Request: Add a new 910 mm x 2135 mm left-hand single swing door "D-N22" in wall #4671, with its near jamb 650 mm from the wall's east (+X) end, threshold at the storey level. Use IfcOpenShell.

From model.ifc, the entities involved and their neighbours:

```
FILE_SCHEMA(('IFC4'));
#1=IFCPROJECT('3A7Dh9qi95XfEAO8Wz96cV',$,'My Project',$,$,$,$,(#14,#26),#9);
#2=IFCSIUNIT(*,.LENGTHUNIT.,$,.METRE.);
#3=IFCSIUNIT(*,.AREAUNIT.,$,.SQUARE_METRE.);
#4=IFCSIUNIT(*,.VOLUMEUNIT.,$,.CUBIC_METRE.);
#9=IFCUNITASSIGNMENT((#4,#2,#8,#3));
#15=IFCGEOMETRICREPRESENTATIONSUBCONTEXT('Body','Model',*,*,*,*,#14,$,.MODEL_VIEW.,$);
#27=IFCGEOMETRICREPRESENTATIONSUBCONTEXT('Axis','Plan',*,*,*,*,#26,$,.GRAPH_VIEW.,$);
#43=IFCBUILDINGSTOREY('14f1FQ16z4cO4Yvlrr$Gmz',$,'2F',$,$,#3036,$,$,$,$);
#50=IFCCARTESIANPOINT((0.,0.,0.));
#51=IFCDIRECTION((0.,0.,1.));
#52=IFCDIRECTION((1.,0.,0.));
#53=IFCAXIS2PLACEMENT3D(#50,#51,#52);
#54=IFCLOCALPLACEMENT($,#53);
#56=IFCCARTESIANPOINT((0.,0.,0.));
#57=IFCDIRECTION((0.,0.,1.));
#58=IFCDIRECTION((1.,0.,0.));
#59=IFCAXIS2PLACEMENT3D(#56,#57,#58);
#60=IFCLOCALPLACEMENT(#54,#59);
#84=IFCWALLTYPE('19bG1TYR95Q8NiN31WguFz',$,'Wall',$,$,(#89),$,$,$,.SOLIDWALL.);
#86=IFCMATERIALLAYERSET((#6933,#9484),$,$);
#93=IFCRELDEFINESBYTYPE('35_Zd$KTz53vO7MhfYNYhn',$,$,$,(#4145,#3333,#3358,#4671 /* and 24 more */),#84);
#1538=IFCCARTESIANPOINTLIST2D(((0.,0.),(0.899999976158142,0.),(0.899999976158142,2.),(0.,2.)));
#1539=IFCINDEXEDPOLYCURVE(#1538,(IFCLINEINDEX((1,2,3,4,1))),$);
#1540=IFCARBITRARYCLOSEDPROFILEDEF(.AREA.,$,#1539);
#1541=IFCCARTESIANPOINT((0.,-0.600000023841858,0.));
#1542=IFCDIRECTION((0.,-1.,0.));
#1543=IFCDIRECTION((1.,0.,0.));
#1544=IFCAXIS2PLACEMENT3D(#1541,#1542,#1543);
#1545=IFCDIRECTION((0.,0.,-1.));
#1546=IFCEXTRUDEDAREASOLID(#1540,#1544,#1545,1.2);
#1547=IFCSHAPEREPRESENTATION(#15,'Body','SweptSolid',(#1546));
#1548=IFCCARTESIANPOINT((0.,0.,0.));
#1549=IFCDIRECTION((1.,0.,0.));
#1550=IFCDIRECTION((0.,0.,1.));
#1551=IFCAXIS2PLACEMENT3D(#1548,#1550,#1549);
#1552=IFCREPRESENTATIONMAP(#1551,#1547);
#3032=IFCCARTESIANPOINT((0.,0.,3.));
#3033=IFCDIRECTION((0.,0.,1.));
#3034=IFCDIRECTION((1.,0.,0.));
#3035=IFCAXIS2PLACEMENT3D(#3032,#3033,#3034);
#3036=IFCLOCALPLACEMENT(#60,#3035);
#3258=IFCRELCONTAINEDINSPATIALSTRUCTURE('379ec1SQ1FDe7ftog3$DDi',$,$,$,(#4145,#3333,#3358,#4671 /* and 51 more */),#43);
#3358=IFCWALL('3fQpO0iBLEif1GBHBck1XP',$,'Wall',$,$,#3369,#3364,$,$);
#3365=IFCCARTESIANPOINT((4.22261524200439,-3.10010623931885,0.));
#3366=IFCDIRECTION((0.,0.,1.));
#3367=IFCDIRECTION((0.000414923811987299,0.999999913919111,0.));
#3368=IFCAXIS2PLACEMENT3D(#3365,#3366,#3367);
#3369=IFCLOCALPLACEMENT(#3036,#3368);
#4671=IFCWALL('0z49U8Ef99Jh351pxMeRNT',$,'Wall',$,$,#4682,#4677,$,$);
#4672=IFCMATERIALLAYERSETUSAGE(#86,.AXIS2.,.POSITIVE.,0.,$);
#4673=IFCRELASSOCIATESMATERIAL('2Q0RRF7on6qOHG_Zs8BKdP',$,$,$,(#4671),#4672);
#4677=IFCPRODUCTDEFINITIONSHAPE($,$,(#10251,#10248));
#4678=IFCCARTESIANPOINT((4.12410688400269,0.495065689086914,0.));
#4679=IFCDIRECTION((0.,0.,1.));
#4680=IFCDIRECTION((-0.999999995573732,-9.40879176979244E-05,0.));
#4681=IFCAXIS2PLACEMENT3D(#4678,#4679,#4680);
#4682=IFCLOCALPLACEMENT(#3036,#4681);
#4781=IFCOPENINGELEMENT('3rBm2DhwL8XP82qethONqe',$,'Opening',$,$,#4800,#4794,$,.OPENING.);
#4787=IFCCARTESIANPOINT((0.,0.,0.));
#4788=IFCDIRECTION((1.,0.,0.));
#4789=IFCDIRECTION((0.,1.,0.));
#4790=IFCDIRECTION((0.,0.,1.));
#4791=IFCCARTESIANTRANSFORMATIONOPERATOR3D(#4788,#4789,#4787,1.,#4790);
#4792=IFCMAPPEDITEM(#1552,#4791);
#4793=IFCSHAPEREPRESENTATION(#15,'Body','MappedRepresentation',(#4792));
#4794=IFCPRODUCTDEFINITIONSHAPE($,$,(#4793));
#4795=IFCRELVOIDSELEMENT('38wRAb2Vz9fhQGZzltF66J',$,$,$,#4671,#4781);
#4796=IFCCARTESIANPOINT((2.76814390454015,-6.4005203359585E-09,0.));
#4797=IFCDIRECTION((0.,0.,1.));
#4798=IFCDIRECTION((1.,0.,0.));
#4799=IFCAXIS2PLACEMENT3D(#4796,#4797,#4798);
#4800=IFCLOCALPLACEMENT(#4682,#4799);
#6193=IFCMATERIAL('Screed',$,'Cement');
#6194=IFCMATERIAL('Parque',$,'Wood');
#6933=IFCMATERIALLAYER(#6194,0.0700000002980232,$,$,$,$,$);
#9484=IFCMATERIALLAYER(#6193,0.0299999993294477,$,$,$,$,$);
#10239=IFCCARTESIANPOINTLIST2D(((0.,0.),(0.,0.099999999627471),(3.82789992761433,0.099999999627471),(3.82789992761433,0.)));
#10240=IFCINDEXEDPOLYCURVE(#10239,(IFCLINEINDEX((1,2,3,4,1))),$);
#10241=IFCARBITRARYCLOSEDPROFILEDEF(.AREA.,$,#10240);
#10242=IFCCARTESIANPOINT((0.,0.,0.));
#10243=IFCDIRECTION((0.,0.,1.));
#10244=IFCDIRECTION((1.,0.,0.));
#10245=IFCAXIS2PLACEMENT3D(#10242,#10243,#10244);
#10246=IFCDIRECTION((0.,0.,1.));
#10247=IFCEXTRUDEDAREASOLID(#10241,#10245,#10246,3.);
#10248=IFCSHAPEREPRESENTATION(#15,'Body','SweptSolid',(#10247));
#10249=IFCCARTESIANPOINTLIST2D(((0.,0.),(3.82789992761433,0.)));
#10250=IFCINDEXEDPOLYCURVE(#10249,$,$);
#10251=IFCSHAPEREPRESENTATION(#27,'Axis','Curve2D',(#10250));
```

```python
import numpy as np
import ifcopenshell
import ifcopenshell.api.feature
import ifcopenshell.api.geometry
import ifcopenshell.api.root
import ifcopenshell.api.spatial
import ifcopenshell.geom
import ifcopenshell.util.element
import ifcopenshell.util.placement
import ifcopenshell.util.representation
import ifcopenshell.util.shape
import ifcopenshell.util.unit

model = ifcopenshell.open("model.ifc")
unit_scale = ifcopenshell.util.unit.calculate_unit_scale(model)
settings = ifcopenshell.geom.settings()


def volume(element):
    """Net volume in cubic metres, openings subtracted."""
    shape = ifcopenshell.geom.create_shape(settings, element)
    return ifcopenshell.util.shape.get_volume(shape.geometry)


wall = model.by_guid("0z49U8Ef99Jh351pxMeRNT")
storey = ifcopenshell.util.element.get_container(wall, ifc_class="IfcBuildingStorey")
context = ifcopenshell.util.representation.get_context(model, "Model", "Body", "MODEL_VIEW")
before = volume(wall)

width, height, from_end, sill = 0.91, 2.135, 0.65, 0.0  # metres

# The wall runs along its own X axis, and the end named is its -X end.
wall_shape = ifcopenshell.geom.create_shape(settings, wall)
x, y, z = ifcopenshell.util.shape.get_vertices(wall_shape.geometry).T
start = x.min() + from_end
face, thickness = float(y.min()), float(y.max() - y.min())
wall_matrix = ifcopenshell.util.placement.get_local_placement(wall.ObjectPlacement)
level = ifcopenshell.util.placement.get_local_placement(storey.ObjectPlacement)[2, 3]


def in_wall(x, y):
    """Placement at x, y metres in the wall's axes, at sill height."""
    matrix = wall_matrix.copy()
    matrix[:, 3] = wall_matrix @ np.array([x / unit_scale, y / unit_scale, 0.0, 1.0])
    matrix[2, 3] = level + sill / unit_scale
    return matrix


# Opening: a box that overshoots both wall faces by 50 mm.
opening = ifcopenshell.api.root.create_entity(model, ifc_class="IfcOpeningElement", predefined_type="OPENING")
box = ifcopenshell.api.geometry.add_wall_representation(
    model, context=context, length=width, height=height, thickness=thickness + 0.1
)
ifcopenshell.api.geometry.assign_representation(model, product=opening, representation=box)
ifcopenshell.api.geometry.edit_object_placement(model, product=opening, matrix=in_wall(start, face - 0.05), is_si=False)
ifcopenshell.api.feature.add_feature(model, feature=opening, element=wall)

door = ifcopenshell.api.root.create_entity(model, ifc_class="IfcDoor", name="D-N22", predefined_type="DOOR")
door.OverallWidth, door.OverallHeight = width / unit_scale, height / unit_scale
door.OperationType = "SINGLE_SWING_LEFT"
body = ifcopenshell.api.geometry.add_door_representation(
    model,
    context=context,
    overall_width=door.OverallWidth,
    overall_height=door.OverallHeight,
    operation_type="SINGLE_SWING_LEFT",
    lining_properties={"LiningDepth": thickness / unit_scale, "ThresholdDepth": thickness / unit_scale},
)
ifcopenshell.api.geometry.assign_representation(model, product=door, representation=body)
ifcopenshell.api.spatial.assign_container(model, products=[door], relating_structure=storey)
ifcopenshell.api.feature.add_filling(model, opening=opening, element=door)

# The lining spans the wall, so the door starts at the wall face.
ifcopenshell.api.geometry.edit_object_placement(model, product=door, matrix=in_wall(start, face), is_si=False)

after = volume(wall)

print(f"wall volume {before:.3f} -> {after:.3f} m3")

model.write("model-out.ifc")
```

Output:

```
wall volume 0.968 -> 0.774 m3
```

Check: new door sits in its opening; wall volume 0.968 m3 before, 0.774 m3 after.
